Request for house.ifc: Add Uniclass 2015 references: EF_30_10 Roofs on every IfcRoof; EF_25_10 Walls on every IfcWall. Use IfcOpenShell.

First a look at what the model holds.

```python
import ifcopenshell

model = ifcopenshell.open("house.ifc")
print(model.schema)
print("classifications:", [c.Name for c in model.by_type("IfcClassification")])
for ifc_class in ("IfcDoor", "IfcRoof", "IfcStair", "IfcWall", "IfcWindow"):
    print(ifc_class, len(model.by_type(ifc_class)))
```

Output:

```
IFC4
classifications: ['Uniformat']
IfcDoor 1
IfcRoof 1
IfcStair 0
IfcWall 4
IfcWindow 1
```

```python
import ifcopenshell
import ifcopenshell.api.classification

model = ifcopenshell.open("house.ifc")

system = ifcopenshell.api.classification.add_classification(model, classification="Uniclass 2015")

codes = {
    "IfcRoof": ("EF_30_10", "Roofs"),
    "IfcWall": ("EF_25_10", "Walls"),
}
for ifc_class, (code, name) in codes.items():
    products = model.by_type(ifc_class)
    ifcopenshell.api.classification.add_reference(
        model, products=products, classification=system, identification=code, name=name
    )
    print(code, len(products))

model.write("house_updated.ifc")
```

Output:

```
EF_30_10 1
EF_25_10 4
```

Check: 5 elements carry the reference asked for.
